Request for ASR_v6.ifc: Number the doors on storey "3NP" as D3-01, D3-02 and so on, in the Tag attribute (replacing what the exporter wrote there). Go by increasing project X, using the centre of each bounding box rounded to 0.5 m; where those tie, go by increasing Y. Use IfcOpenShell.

First a look at what the model holds.

```python
import ifcopenshell
import ifcopenshell.util.element
import ifcopenshell.util.placement

model = ifcopenshell.open("ASR_v6.ifc")
print(model.schema)
storey = next(s for s in model.by_type("IfcBuildingStorey") if s.Name == "3NP")
doors = [e for e in ifcopenshell.util.element.get_decomposition(storey) if e.is_a("IfcDoor")]
for e in sorted(doors, key=lambda e: e.id()):
    origin = ifcopenshell.util.placement.get_local_placement(e.ObjectPlacement)[:3, 3]
    print(e.id(), e.Tag, e.Name, origin.round(2) + 0.0, sep=" | ")
```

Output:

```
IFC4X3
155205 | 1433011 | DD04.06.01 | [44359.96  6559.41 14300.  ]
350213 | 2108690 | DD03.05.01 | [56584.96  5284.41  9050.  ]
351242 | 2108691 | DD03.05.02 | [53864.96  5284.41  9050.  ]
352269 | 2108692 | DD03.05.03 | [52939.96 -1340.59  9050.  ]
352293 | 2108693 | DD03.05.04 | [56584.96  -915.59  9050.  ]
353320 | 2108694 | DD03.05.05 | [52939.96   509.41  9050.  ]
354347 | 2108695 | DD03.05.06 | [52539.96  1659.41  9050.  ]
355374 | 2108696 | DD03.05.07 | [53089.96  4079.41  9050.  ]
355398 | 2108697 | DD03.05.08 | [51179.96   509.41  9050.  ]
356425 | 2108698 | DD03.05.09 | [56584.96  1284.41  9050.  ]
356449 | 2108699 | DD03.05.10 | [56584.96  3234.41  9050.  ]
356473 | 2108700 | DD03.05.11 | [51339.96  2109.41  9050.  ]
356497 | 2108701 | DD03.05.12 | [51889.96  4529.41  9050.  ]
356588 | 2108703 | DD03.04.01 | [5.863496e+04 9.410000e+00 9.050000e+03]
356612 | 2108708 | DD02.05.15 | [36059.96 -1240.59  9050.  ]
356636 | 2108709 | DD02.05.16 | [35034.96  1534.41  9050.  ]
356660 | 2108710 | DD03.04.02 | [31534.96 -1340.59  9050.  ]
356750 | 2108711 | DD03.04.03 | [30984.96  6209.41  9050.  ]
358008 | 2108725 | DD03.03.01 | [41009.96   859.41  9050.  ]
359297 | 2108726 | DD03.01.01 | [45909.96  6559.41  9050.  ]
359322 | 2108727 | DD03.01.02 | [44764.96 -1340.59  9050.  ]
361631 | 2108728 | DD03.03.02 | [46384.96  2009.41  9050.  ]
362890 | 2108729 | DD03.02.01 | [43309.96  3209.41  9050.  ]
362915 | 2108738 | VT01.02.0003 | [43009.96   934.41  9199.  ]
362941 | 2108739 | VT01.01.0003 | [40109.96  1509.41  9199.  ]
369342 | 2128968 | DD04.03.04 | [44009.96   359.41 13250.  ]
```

```python
import ifcopenshell
import ifcopenshell.geom
import ifcopenshell.util.element
import ifcopenshell.util.shape

model = ifcopenshell.open("ASR_v6.ifc")
settings = ifcopenshell.geom.settings()
settings.set("use-world-coords", True)


def centre(element):
    shape = ifcopenshell.geom.create_shape(settings, element)
    return ifcopenshell.util.shape.get_bbox_centroid(shape.geometry)


storey = next(s for s in model.by_type("IfcBuildingStorey") if s.Name == "3NP")
doors = [e for e in ifcopenshell.util.element.get_decomposition(storey) if e.is_a("IfcDoor")]

# Insertion points can sit at a corner or the storey origin, so sort by the geometry (in metres).
centres = {e: centre(e) for e in doors}
doors.sort(key=lambda e: (round(centres[e][0] / 0.5), centres[e][1]))

for i, e in enumerate(doors, start=1):
    number = f"D3-{i:02d}"
    e.Tag = number
    print(e.id(), number)

model.write("ASR_v6_edited.ifc")
```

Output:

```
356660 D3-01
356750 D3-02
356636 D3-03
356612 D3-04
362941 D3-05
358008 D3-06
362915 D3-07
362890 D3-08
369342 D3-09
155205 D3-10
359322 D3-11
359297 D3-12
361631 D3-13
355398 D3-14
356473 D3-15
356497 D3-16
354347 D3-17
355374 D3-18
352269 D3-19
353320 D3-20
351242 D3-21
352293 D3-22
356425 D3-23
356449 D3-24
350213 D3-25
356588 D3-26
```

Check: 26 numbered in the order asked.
